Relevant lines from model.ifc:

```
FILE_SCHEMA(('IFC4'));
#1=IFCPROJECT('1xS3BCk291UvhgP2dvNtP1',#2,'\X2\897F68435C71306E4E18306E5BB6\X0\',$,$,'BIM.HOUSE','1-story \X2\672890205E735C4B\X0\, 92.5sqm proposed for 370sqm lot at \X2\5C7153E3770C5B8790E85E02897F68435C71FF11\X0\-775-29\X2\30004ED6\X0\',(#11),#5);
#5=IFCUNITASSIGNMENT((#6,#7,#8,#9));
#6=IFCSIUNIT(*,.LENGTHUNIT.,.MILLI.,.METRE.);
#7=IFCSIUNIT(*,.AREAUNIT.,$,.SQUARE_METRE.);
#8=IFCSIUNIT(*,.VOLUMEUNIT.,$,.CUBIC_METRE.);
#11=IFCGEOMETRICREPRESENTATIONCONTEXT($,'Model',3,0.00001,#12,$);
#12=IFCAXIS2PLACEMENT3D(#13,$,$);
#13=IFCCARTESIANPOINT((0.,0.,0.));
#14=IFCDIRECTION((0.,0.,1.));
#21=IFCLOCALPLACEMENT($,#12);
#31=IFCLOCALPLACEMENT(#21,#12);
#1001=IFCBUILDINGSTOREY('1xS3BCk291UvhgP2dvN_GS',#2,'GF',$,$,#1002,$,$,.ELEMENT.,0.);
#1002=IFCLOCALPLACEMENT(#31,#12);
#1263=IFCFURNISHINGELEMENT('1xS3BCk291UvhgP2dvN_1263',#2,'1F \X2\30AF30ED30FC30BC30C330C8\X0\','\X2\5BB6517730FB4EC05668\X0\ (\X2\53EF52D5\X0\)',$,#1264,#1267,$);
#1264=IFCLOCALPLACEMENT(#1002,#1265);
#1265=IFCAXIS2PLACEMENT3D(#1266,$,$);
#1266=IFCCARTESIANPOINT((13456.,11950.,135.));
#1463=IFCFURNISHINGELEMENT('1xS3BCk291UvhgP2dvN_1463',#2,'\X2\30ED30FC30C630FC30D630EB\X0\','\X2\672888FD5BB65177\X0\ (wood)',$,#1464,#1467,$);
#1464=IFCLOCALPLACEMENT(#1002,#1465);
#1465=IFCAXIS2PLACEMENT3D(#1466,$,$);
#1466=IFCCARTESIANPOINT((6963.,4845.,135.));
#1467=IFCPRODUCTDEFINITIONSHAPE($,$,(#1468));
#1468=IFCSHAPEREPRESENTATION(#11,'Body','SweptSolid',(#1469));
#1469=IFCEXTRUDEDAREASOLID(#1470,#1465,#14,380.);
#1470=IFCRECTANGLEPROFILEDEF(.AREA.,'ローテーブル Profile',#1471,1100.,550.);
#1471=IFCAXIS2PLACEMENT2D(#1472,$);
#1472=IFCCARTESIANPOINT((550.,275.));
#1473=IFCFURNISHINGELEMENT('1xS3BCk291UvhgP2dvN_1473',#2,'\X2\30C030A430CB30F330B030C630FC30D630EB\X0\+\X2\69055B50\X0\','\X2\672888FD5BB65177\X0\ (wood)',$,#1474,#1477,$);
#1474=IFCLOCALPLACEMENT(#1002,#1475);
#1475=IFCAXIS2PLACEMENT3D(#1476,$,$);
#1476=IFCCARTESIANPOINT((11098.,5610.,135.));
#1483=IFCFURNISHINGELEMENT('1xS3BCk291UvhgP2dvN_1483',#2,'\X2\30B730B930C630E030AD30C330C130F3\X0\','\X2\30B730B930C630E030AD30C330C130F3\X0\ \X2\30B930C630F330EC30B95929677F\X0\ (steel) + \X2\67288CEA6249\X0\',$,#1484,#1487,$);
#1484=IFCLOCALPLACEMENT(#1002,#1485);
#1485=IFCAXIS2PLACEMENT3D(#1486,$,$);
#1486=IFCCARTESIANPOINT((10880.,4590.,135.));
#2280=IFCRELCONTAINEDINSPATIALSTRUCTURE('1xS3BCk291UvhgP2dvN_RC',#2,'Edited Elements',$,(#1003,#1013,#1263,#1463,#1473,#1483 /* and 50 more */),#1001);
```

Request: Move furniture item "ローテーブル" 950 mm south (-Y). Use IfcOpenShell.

```python
import ifcopenshell
import ifcopenshell.api.geometry
import ifcopenshell.util.placement
import ifcopenshell.util.unit

model = ifcopenshell.open("model.ifc")
unit_scale = ifcopenshell.util.unit.calculate_unit_scale(model)

item = model.by_guid("1xS3BCk291UvhgP2dvN_1463")
matrix = ifcopenshell.util.placement.get_local_placement(item.ObjectPlacement)
matrix[1, 3] -= 0.95 / unit_scale
ifcopenshell.api.geometry.edit_object_placement(model, product=item, matrix=matrix, is_si=False)

print(ifcopenshell.util.placement.get_local_placement(item.ObjectPlacement).round(3) + 0.0)

model.write("model-out.ifc")
```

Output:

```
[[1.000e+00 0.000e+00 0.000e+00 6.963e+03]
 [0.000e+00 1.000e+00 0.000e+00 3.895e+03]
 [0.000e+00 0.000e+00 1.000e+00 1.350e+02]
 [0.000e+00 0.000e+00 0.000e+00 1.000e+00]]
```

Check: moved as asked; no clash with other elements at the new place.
